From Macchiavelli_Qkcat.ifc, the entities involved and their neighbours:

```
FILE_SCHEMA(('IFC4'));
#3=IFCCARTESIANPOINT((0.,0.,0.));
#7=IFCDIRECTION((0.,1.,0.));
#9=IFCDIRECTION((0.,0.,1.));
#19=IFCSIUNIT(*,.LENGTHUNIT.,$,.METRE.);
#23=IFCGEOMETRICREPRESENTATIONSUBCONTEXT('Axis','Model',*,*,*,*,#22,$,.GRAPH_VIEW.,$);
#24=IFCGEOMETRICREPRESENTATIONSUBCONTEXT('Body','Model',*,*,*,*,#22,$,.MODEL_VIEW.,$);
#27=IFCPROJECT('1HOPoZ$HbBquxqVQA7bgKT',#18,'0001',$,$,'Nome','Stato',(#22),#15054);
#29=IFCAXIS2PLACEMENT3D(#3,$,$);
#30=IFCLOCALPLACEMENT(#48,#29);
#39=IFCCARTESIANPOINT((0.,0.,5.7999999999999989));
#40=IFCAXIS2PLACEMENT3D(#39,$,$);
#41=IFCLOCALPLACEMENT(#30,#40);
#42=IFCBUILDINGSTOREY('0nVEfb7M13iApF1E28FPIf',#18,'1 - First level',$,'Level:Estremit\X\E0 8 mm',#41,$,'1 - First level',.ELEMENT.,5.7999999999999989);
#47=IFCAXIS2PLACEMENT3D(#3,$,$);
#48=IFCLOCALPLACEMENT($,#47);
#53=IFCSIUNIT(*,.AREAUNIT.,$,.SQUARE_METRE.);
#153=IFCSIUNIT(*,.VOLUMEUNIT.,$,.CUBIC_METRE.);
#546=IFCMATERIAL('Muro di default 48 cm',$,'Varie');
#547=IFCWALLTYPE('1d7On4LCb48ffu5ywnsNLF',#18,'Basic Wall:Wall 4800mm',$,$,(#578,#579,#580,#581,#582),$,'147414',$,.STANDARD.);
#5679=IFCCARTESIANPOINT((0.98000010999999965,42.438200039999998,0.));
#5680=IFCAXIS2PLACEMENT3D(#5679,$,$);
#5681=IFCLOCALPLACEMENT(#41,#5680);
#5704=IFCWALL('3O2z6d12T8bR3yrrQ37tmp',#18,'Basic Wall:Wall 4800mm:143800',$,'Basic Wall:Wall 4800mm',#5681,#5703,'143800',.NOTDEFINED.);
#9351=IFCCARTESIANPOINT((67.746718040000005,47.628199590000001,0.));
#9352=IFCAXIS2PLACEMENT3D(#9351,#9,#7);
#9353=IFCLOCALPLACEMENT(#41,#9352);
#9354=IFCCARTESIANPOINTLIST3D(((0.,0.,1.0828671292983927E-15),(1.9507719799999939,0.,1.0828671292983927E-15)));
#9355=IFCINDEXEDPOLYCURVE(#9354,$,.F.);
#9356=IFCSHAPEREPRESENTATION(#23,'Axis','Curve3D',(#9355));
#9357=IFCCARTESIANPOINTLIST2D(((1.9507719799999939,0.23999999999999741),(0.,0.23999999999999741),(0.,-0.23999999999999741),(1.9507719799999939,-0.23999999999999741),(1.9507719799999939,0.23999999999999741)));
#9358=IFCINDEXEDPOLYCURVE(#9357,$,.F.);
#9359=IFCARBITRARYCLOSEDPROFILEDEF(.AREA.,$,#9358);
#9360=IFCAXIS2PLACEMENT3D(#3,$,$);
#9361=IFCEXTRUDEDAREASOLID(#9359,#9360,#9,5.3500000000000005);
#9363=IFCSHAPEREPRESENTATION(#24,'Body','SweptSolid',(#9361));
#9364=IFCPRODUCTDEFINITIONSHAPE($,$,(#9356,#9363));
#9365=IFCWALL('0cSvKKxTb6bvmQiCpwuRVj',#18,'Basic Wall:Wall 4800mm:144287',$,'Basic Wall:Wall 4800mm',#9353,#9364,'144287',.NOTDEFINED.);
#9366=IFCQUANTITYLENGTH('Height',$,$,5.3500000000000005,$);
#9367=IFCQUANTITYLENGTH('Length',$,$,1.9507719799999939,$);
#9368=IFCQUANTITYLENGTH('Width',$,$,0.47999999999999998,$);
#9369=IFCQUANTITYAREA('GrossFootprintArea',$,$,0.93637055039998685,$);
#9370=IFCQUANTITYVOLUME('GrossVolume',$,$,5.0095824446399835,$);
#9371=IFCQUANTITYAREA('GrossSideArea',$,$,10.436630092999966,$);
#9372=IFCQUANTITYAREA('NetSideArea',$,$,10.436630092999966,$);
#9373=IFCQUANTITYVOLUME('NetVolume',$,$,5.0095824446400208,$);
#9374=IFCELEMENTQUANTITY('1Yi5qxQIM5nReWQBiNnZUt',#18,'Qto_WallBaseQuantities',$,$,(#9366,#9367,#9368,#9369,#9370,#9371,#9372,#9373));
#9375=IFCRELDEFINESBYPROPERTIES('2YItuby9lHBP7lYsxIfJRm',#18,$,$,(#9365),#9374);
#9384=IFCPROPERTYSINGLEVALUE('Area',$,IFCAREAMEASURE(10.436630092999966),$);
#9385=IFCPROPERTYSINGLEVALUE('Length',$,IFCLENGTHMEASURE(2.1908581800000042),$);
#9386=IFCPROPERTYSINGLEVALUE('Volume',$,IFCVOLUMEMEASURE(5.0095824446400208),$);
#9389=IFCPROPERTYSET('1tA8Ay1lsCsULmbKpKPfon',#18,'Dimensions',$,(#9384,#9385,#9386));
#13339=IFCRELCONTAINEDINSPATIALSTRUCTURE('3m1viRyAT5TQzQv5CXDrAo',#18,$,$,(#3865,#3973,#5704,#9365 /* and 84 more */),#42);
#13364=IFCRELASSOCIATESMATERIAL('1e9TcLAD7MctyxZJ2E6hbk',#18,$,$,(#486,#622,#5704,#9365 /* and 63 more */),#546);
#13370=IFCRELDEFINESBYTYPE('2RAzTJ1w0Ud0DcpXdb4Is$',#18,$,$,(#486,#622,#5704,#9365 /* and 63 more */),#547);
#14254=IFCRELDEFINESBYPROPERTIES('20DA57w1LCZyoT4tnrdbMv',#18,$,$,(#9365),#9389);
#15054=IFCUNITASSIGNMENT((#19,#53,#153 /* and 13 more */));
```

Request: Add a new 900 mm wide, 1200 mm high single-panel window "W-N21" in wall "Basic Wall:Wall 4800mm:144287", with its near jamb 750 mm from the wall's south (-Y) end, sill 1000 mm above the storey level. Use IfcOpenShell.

```python
import numpy as np
import ifcopenshell
import ifcopenshell.api.feature
import ifcopenshell.api.geometry
import ifcopenshell.api.pset
import ifcopenshell.api.root
import ifcopenshell.api.spatial
import ifcopenshell.geom
import ifcopenshell.util.element
import ifcopenshell.util.placement
import ifcopenshell.util.representation
import ifcopenshell.util.shape
import ifcopenshell.util.unit

model = ifcopenshell.open("Macchiavelli_Qkcat.ifc")
unit_scale = ifcopenshell.util.unit.calculate_unit_scale(model)
area_scale = ifcopenshell.util.unit.calculate_unit_scale(model, "AREAUNIT")
volume_scale = ifcopenshell.util.unit.calculate_unit_scale(model, "VOLUMEUNIT")
settings = ifcopenshell.geom.settings()


def volume(element):
    """Net volume in cubic metres, openings subtracted."""
    shape = ifcopenshell.geom.create_shape(settings, element)
    return ifcopenshell.util.shape.get_volume(shape.geometry)


wall = model.by_id(9365)
storey = ifcopenshell.util.element.get_container(wall, ifc_class="IfcBuildingStorey")
context = ifcopenshell.util.representation.get_context(model, "Model", "Body", "MODEL_VIEW")
before = volume(wall)

width, height, from_end, sill = 0.9, 1.2, 0.75, 1  # metres

# The wall runs along its own X axis, and the end named is its -X end.
wall_shape = ifcopenshell.geom.create_shape(settings, wall)
x, y, z = ifcopenshell.util.shape.get_vertices(wall_shape.geometry).T
start = x.min() + from_end
face, thickness = float(y.min()), float(y.max() - y.min())
wall_matrix = ifcopenshell.util.placement.get_local_placement(wall.ObjectPlacement)
level = ifcopenshell.util.placement.get_local_placement(storey.ObjectPlacement)[2, 3]


def in_wall(x, y):
    """Placement at x, y metres in the wall's axes, at sill height."""
    matrix = wall_matrix.copy()
    matrix[:, 3] = wall_matrix @ np.array([x / unit_scale, y / unit_scale, 0.0, 1.0])
    matrix[2, 3] = level + sill / unit_scale
    return matrix


# Opening: a box that overshoots both wall faces by 50 mm.
opening = ifcopenshell.api.root.create_entity(model, ifc_class="IfcOpeningElement", predefined_type="OPENING")
box = ifcopenshell.api.geometry.add_wall_representation(
    model, context=context, length=width, height=height, thickness=thickness + 0.1
)
ifcopenshell.api.geometry.assign_representation(model, product=opening, representation=box)
ifcopenshell.api.geometry.edit_object_placement(model, product=opening, matrix=in_wall(start, face - 0.05), is_si=False)
ifcopenshell.api.feature.add_feature(model, feature=opening, element=wall)

window = ifcopenshell.api.root.create_entity(model, ifc_class="IfcWindow", name="W-N21", predefined_type="WINDOW")
window.OverallWidth, window.OverallHeight = width / unit_scale, height / unit_scale
window.PartitioningType = "SINGLE_PANEL"
body = ifcopenshell.api.geometry.add_window_representation(
    model,
    context=context,
    overall_width=window.OverallWidth,
    overall_height=window.OverallHeight,
    partition_type="SINGLE_PANEL",
)
ifcopenshell.api.geometry.assign_representation(model, product=window, representation=body)
ifcopenshell.api.spatial.assign_container(model, products=[window], relating_structure=storey)
ifcopenshell.api.feature.add_filling(model, opening=opening, element=window)

# Centre the window in the wall's thickness.
ifcopenshell.api.geometry.edit_object_placement(model, product=window, matrix=in_wall(start, face), is_si=False)
window_shape = ifcopenshell.geom.create_shape(settings, window)
depth = ifcopenshell.util.shape.get_vertices(window_shape.geometry)[:, 1]
offset = face + thickness / 2 - (depth.min() + depth.max()) / 2
ifcopenshell.api.geometry.edit_object_placement(model, product=window, matrix=in_wall(start, offset), is_si=False)

after = volume(wall)

# Update the wall's stored quantities.
qto = model.by_id(ifcopenshell.util.element.get_pset(wall, "Qto_WallBaseQuantities", should_inherit=False)["id"])
ifcopenshell.api.pset.edit_qto(model, qto=qto, properties={
    "NetSideArea": after / thickness / area_scale,
    "NetVolume": after / volume_scale,
})
pset = model.by_id(ifcopenshell.util.element.get_pset(wall, "Dimensions", should_inherit=False)["id"])
ifcopenshell.api.pset.edit_pset(model, pset=pset, properties={
    "Area": model.create_entity("IfcAreaMeasure", after / thickness / area_scale),
    "Volume": model.create_entity("IfcVolumeMeasure", after / volume_scale),
})

print(f"wall volume {before:.3f} -> {after:.3f} m3")

model.write("Macchiavelli_Qkcat_edited.ifc")
```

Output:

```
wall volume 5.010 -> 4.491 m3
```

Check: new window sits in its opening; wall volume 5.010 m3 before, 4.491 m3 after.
